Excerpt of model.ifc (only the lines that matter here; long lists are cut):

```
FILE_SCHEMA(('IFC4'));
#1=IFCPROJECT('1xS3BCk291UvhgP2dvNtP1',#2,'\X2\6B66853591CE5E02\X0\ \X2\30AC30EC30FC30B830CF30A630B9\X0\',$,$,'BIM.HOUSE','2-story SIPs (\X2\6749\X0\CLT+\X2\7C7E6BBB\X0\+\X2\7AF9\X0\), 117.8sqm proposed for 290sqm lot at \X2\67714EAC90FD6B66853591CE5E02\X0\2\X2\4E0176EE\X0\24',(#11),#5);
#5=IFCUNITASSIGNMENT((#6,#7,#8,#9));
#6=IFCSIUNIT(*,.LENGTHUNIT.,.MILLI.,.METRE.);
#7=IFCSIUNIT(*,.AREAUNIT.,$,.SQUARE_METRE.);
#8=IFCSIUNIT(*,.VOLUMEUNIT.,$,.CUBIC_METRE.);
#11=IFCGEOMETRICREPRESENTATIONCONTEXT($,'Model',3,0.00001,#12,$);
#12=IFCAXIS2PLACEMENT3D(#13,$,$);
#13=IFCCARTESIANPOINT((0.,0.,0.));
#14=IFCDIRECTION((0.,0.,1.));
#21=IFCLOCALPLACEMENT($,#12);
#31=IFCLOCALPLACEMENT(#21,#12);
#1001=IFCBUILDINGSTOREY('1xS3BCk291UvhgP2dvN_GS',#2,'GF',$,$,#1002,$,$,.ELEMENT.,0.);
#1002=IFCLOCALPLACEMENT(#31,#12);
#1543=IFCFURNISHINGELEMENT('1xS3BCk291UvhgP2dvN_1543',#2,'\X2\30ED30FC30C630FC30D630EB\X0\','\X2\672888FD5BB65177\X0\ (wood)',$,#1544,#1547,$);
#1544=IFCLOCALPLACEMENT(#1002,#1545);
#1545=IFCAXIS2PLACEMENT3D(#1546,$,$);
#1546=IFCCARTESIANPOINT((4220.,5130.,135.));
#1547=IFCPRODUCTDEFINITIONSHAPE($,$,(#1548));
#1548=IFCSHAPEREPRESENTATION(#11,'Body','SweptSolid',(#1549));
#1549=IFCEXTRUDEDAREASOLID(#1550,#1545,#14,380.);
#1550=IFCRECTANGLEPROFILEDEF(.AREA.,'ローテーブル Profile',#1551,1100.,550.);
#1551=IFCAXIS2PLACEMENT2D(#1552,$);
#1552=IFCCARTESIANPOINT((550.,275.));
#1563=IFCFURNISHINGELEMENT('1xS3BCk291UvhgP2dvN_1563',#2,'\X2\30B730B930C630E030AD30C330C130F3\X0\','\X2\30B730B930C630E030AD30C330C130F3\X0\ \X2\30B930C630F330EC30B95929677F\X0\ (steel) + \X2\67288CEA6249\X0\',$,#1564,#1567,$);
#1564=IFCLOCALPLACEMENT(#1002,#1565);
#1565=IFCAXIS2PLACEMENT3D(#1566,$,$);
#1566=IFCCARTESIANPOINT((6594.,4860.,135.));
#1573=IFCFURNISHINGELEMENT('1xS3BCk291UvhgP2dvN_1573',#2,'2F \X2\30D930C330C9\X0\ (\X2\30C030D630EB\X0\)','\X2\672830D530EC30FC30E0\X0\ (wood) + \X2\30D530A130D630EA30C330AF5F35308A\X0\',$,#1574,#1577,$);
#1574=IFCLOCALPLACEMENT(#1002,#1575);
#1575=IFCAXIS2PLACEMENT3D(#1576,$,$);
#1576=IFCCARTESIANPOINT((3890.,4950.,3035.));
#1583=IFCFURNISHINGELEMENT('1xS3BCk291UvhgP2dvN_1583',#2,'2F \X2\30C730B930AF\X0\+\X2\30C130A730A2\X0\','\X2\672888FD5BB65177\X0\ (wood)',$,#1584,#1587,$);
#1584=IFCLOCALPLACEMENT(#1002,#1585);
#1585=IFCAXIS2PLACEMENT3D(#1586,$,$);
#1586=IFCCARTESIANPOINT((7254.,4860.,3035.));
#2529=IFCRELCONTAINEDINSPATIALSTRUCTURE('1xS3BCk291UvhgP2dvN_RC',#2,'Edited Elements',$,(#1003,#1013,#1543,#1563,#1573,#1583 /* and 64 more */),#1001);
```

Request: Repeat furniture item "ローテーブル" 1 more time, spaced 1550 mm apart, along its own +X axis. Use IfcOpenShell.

```python
import ifcopenshell
import ifcopenshell.api.geometry
import ifcopenshell.api.root
import ifcopenshell.util.element
import ifcopenshell.util.placement
import ifcopenshell.util.unit

model = ifcopenshell.open("model.ifc")
unit_scale = ifcopenshell.util.unit.calculate_unit_scale(model)


def reuse_history(source, copy):
    """copy_class also copies each property set's owner history, people and application; keep the originals."""
    for rel in copy.IsDefinedBy:
        if rel.is_a("IfcRelDefinesByProperties") and (history := rel.RelatingPropertyDefinition.OwnerHistory):
            rel.RelatingPropertyDefinition.OwnerHistory = source.OwnerHistory
            ifcopenshell.util.element.remove_deep2(model, history)


source = model.by_id(1543)
base = ifcopenshell.util.placement.get_local_placement(source.ObjectPlacement)
step = base[:3, 0] * 1.55 / unit_scale

for i in range(1, 2):
    copy = ifcopenshell.api.root.copy_class(model, product=source)
    copy.Representation = ifcopenshell.util.element.copy_deep(
        model, source.Representation, exclude=["IfcGeometricRepresentationContext", "IfcRepresentationMap"]
    )
    reuse_history(source, copy)
    matrix = base.copy()
    matrix[:3, 3] += i * step
    print("added at", matrix[:3, 3].round(3) + 0.0)
    ifcopenshell.api.geometry.edit_object_placement(model, product=copy, matrix=matrix, is_si=False)

model.write("model_v2.ifc")
```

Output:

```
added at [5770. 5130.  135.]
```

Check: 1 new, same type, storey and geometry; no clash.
